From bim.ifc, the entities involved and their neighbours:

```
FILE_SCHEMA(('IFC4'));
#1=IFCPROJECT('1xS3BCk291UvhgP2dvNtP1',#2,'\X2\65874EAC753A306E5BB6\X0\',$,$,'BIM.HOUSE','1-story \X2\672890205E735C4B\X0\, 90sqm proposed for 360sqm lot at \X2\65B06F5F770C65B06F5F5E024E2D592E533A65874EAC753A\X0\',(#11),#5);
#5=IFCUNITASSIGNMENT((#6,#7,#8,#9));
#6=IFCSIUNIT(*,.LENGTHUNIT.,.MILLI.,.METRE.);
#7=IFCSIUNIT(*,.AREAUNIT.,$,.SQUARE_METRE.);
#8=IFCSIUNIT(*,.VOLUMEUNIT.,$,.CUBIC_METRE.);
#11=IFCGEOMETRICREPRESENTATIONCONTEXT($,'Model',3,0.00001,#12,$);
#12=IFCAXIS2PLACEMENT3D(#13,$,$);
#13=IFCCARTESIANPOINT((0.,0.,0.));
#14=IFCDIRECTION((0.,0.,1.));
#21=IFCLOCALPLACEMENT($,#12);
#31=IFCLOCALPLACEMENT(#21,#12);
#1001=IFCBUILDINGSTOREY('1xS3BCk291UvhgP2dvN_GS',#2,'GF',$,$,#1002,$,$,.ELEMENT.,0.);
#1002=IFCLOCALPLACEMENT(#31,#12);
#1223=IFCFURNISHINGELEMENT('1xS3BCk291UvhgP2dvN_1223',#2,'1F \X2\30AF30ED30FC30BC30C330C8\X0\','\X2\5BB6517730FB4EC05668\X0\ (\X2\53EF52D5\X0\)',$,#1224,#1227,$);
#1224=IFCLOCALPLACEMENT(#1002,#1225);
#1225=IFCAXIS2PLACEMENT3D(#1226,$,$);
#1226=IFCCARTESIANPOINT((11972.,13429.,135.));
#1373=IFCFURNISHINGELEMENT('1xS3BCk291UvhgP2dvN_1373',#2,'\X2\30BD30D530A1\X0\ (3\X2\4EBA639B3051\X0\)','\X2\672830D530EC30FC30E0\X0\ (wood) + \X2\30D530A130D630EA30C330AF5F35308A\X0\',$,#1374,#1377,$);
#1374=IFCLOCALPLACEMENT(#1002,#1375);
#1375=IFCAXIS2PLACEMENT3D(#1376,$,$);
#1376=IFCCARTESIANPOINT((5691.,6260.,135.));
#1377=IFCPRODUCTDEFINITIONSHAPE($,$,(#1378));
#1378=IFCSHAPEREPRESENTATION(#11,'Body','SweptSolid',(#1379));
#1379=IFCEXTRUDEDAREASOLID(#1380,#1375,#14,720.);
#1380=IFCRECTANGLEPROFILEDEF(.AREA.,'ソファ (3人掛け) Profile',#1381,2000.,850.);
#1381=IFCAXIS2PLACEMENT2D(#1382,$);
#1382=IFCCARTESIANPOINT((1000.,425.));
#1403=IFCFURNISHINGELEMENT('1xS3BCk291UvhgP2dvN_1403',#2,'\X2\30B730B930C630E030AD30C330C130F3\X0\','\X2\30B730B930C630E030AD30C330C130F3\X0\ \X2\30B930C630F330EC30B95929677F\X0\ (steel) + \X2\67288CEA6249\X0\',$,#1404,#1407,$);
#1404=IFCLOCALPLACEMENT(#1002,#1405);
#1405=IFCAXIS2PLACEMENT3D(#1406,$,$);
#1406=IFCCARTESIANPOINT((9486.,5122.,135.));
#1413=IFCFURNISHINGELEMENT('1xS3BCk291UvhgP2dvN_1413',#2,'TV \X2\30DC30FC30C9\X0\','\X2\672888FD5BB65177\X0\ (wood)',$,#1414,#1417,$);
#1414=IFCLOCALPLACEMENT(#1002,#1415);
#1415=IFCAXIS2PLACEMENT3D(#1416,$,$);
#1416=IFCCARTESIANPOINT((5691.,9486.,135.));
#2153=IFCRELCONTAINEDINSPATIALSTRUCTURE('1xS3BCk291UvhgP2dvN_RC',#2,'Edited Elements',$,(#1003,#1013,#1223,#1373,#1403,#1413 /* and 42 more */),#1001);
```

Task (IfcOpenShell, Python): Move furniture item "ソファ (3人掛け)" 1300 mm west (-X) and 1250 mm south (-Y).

```python
import ifcopenshell
import ifcopenshell.api.geometry
import ifcopenshell.util.placement
import ifcopenshell.util.unit

model = ifcopenshell.open("bim.ifc")
unit_scale = ifcopenshell.util.unit.calculate_unit_scale(model)

item = model.by_guid("1xS3BCk291UvhgP2dvN_1373")
matrix = ifcopenshell.util.placement.get_local_placement(item.ObjectPlacement)
matrix[0, 3] -= 1.3 / unit_scale
matrix[1, 3] -= 1.25 / unit_scale
ifcopenshell.api.geometry.edit_object_placement(model, product=item, matrix=matrix, is_si=False)

print(ifcopenshell.util.placement.get_local_placement(item.ObjectPlacement).round(3) + 0.0)

model.write("bim_edited.ifc")
```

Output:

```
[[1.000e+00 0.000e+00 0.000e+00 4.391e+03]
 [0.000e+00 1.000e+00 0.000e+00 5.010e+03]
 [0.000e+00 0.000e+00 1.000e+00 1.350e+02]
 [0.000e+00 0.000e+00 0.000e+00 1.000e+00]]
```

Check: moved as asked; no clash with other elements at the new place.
